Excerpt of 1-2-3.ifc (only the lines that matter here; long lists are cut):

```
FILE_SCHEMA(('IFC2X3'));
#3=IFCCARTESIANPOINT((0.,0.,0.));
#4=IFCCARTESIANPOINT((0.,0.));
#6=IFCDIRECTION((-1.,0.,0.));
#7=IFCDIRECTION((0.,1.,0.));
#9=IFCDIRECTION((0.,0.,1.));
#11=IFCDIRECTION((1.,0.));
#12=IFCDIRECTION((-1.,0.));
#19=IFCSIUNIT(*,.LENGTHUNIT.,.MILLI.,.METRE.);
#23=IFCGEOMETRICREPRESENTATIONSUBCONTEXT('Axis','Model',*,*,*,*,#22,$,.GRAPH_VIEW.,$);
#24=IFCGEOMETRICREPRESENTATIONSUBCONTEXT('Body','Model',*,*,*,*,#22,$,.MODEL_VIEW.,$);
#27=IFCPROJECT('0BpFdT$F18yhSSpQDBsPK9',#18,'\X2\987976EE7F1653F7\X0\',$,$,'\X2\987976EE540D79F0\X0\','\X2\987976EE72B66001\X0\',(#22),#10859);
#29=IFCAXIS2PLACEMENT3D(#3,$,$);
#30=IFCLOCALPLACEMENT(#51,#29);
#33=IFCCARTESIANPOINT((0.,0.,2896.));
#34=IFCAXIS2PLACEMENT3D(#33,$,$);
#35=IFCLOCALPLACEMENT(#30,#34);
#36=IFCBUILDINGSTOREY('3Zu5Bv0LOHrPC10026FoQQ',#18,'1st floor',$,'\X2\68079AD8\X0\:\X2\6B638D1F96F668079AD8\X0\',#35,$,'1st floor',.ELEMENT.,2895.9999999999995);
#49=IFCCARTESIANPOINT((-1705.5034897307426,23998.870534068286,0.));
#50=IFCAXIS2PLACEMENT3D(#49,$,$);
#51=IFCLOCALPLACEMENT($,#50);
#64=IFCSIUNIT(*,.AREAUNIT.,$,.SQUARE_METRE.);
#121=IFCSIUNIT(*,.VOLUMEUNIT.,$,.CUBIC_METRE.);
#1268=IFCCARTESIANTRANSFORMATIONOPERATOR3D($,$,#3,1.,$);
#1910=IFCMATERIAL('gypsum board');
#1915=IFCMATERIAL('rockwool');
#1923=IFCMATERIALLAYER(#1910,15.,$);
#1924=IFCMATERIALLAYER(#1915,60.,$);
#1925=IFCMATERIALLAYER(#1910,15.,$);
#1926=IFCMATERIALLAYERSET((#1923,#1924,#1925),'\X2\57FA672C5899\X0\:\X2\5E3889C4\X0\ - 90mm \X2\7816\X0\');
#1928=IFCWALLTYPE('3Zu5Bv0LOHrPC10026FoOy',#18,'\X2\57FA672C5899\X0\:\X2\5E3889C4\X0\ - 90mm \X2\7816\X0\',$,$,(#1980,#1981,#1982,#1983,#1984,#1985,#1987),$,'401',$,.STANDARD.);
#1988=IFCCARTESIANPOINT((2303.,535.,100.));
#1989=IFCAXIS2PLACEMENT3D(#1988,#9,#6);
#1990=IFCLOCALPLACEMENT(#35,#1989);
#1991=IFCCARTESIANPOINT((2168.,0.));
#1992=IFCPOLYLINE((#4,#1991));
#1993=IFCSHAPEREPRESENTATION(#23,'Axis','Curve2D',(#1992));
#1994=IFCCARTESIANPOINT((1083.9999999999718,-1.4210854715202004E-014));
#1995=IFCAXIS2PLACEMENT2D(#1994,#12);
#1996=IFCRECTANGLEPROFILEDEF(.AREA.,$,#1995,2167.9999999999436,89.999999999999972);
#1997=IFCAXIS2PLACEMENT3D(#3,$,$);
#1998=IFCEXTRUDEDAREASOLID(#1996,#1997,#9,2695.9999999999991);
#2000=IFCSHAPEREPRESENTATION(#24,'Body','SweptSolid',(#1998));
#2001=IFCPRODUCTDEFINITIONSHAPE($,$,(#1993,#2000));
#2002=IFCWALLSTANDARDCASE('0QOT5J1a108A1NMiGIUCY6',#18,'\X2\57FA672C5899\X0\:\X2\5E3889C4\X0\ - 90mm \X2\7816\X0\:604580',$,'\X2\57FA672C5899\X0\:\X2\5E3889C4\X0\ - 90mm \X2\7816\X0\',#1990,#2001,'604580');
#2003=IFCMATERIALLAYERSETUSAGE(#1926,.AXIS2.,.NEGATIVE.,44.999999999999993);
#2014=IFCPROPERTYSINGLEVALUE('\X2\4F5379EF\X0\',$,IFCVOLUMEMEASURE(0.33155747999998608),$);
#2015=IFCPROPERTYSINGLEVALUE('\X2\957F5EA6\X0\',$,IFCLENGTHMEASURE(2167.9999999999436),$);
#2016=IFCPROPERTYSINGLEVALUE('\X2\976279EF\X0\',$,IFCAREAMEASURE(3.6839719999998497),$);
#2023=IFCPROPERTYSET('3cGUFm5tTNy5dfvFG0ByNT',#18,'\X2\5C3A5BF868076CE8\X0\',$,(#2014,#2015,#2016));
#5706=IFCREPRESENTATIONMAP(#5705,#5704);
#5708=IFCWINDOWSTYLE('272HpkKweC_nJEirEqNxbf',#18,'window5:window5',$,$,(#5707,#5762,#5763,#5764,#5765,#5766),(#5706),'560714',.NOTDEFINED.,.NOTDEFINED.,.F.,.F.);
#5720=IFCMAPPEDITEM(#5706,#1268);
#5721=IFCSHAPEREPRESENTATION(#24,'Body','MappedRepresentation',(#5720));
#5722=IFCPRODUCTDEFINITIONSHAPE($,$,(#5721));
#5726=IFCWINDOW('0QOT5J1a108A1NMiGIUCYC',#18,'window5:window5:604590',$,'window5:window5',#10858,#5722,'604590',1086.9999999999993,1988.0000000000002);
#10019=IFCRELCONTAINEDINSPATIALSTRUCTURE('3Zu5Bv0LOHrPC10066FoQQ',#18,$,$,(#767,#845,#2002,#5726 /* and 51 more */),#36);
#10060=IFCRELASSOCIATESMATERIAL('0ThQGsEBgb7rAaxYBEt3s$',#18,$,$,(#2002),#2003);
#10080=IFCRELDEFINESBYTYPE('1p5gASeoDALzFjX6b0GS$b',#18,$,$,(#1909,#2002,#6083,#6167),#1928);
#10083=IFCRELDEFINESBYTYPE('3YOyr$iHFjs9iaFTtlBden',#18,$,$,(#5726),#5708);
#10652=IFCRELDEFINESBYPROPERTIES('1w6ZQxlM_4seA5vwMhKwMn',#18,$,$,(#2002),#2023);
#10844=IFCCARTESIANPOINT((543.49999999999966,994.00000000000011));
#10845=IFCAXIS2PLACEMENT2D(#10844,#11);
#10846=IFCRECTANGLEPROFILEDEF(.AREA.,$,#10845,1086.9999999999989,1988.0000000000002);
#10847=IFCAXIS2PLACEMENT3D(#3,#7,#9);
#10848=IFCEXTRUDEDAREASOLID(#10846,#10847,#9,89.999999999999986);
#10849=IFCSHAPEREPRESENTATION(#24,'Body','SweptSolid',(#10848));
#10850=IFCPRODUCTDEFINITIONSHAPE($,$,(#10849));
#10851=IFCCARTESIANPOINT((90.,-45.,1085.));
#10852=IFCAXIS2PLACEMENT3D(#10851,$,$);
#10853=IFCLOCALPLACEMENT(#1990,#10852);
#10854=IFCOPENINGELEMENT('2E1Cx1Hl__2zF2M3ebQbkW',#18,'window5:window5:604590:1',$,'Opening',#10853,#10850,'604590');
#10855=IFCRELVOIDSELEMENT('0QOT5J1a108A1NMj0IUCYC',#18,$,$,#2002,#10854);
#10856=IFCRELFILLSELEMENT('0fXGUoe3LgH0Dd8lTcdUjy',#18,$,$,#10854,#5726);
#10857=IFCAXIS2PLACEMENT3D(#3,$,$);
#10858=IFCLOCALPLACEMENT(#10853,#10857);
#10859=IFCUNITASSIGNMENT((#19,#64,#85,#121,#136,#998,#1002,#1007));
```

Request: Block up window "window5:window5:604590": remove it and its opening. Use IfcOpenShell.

```python
import ifcopenshell
import ifcopenshell.api.feature
import ifcopenshell.api.pset
import ifcopenshell.api.root
import ifcopenshell.geom
import ifcopenshell.util.element
import ifcopenshell.util.shape
import ifcopenshell.util.unit

model = ifcopenshell.open("1-2-3.ifc")
area_scale = ifcopenshell.util.unit.calculate_unit_scale(model, "AREAUNIT")
volume_scale = ifcopenshell.util.unit.calculate_unit_scale(model, "VOLUMEUNIT")
settings = ifcopenshell.geom.settings()


def volume(element):
    """Net volume in cubic metres, openings subtracted."""
    shape = ifcopenshell.geom.create_shape(settings, element)
    return ifcopenshell.util.shape.get_volume(shape.geometry)


window = model.by_id(5726)
opening = window.FillsVoids[0].RelatingOpeningElement
wall = opening.VoidsElements[0].RelatingBuildingElement
before = volume(wall)

ifcopenshell.api.root.remove_product(model, product=window)
ifcopenshell.api.feature.remove_feature(model, feature=opening)

after = volume(wall)
thickness = 0.09  # wall thickness in metres

# Update the wall's stored quantities.
pset = model.by_id(ifcopenshell.util.element.get_pset(wall, "尺寸标注", should_inherit=False)["id"])
ifcopenshell.api.pset.edit_pset(model, pset=pset, properties={
    "体积": model.create_entity("IfcVolumeMeasure", after / volume_scale),
    "面积": model.create_entity("IfcAreaMeasure", after / thickness / area_scale),
})

print(f"wall volume {before:.3f} -> {after:.3f} m3")

model.write("1-2-3_edited.ifc")
```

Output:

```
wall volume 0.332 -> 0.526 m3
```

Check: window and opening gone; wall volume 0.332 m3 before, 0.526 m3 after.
